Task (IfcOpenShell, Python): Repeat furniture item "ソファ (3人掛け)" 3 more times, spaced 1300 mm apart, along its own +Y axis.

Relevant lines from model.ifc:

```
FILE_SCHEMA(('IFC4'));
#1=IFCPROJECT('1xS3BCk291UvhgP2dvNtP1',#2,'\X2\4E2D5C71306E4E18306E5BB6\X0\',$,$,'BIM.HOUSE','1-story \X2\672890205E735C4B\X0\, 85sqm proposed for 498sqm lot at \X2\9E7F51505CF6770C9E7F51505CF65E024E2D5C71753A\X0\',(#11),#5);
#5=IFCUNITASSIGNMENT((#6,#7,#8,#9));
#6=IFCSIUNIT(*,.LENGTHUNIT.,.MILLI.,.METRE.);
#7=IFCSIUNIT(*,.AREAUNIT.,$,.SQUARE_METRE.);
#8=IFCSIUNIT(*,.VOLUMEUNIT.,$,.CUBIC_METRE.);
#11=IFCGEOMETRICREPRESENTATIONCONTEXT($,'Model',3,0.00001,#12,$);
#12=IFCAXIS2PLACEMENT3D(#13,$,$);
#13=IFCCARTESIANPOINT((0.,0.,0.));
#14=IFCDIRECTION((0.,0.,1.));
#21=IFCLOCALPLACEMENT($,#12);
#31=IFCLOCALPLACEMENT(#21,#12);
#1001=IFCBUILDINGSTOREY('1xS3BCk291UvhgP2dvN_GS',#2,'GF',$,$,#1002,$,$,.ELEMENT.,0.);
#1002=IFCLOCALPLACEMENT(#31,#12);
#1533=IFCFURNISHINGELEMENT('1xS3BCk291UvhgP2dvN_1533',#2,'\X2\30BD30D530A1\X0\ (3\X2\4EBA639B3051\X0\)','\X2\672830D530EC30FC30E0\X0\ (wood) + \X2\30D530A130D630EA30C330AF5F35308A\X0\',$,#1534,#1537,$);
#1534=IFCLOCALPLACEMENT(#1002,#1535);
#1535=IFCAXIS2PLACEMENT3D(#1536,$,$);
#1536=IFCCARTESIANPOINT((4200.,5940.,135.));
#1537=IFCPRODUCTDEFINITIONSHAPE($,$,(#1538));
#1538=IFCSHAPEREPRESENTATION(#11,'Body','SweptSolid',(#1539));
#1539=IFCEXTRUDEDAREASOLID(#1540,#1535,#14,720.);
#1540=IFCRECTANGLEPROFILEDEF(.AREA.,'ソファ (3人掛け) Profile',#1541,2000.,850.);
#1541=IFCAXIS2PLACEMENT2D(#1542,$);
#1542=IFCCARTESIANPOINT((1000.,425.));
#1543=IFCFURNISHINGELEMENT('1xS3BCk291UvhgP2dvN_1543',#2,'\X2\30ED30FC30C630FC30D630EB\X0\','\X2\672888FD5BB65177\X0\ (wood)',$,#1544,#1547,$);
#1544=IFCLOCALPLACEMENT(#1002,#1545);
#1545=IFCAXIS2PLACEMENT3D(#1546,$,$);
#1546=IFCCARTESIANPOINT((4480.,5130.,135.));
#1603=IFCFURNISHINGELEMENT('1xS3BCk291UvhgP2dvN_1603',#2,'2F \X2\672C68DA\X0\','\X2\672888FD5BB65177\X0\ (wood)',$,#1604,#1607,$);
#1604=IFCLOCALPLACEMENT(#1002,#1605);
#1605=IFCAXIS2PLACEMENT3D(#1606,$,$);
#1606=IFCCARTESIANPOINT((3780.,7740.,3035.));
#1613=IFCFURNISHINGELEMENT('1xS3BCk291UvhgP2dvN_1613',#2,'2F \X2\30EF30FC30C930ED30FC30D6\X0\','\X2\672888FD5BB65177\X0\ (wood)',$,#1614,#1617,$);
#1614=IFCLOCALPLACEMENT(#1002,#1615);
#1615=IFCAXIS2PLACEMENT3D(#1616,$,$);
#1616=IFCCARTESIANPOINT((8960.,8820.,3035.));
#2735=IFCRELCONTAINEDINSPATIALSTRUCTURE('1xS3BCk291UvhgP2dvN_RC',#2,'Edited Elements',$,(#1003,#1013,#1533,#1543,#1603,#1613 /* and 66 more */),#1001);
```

```python
import ifcopenshell
import ifcopenshell.api.geometry
import ifcopenshell.api.root
import ifcopenshell.util.element
import ifcopenshell.util.placement
import ifcopenshell.util.unit

model = ifcopenshell.open("model.ifc")
unit_scale = ifcopenshell.util.unit.calculate_unit_scale(model)


def reuse_history(source, copy):
    """copy_class also copies each property set's owner history, people and application; keep the originals."""
    for rel in copy.IsDefinedBy:
        if rel.is_a("IfcRelDefinesByProperties") and (history := rel.RelatingPropertyDefinition.OwnerHistory):
            rel.RelatingPropertyDefinition.OwnerHistory = source.OwnerHistory
            ifcopenshell.util.element.remove_deep2(model, history)


source = model.by_guid("1xS3BCk291UvhgP2dvN_1533")
base = ifcopenshell.util.placement.get_local_placement(source.ObjectPlacement)
step = base[:3, 1] * 1.3 / unit_scale

for i in range(1, 4):
    copy = ifcopenshell.api.root.copy_class(model, product=source)
    copy.Representation = ifcopenshell.util.element.copy_deep(
        model, source.Representation, exclude=["IfcGeometricRepresentationContext", "IfcRepresentationMap"]
    )
    reuse_history(source, copy)
    matrix = base.copy()
    matrix[:3, 3] += i * step
    print("added at", matrix[:3, 3].round(3) + 0.0)
    ifcopenshell.api.geometry.edit_object_placement(model, product=copy, matrix=matrix, is_si=False)

model.write("model-out.ifc")
```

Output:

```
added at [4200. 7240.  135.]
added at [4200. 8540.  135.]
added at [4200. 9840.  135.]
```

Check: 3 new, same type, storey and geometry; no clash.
